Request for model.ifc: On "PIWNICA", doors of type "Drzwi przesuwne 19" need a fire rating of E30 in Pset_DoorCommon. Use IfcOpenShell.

First a look at what the model holds.

```python
import ifcopenshell
import ifcopenshell.util.element

model = ifcopenshell.open("model.ifc")
print(model.schema)
storey = next(s for s in model.by_type("IfcBuildingStorey") if s.Name == "PIWNICA")
doors = [e for e in ifcopenshell.util.element.get_decomposition(storey) if e.is_a("IfcDoor")]
seen = {}
for e in doors:
    element_type = ifcopenshell.util.element.get_type(e)
    key = (element_type.Name if element_type != e and element_type else None, ifcopenshell.util.element.get_pset(e, "Pset_DoorCommon", "FireRating"))
    seen[key] = seen.get(key, 0) + 1
for (name, value), count in sorted(seen.items(), key=str):
    print(count, "x", name, "|", value)
```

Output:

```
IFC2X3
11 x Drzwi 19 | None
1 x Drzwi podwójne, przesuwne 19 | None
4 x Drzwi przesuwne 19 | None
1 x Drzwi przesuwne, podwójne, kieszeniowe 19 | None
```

```python
import ifcopenshell
import ifcopenshell.api.pset
import ifcopenshell.util.element

model = ifcopenshell.open("model.ifc")

storey = next(s for s in model.by_type("IfcBuildingStorey") if s.Name == "PIWNICA")
doors = [e for e in ifcopenshell.util.element.get_decomposition(storey) if e.is_a("IfcDoor")]

count = 0
for e in doors:
    element_type = ifcopenshell.util.element.get_type(e)
    if element_type in (None, e) or element_type.Name != "Drzwi przesuwne 19":
        continue
    # add_pset returns the element's existing set when there is one.
    pset = ifcopenshell.api.pset.add_pset(model, product=e, name="Pset_DoorCommon")
    ifcopenshell.api.pset.edit_pset(model, pset=pset, properties={"FireRating": "E30"})
    count += 1

print(count, "doors updated")

model.write("model-out.ifc")
```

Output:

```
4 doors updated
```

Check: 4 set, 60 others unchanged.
